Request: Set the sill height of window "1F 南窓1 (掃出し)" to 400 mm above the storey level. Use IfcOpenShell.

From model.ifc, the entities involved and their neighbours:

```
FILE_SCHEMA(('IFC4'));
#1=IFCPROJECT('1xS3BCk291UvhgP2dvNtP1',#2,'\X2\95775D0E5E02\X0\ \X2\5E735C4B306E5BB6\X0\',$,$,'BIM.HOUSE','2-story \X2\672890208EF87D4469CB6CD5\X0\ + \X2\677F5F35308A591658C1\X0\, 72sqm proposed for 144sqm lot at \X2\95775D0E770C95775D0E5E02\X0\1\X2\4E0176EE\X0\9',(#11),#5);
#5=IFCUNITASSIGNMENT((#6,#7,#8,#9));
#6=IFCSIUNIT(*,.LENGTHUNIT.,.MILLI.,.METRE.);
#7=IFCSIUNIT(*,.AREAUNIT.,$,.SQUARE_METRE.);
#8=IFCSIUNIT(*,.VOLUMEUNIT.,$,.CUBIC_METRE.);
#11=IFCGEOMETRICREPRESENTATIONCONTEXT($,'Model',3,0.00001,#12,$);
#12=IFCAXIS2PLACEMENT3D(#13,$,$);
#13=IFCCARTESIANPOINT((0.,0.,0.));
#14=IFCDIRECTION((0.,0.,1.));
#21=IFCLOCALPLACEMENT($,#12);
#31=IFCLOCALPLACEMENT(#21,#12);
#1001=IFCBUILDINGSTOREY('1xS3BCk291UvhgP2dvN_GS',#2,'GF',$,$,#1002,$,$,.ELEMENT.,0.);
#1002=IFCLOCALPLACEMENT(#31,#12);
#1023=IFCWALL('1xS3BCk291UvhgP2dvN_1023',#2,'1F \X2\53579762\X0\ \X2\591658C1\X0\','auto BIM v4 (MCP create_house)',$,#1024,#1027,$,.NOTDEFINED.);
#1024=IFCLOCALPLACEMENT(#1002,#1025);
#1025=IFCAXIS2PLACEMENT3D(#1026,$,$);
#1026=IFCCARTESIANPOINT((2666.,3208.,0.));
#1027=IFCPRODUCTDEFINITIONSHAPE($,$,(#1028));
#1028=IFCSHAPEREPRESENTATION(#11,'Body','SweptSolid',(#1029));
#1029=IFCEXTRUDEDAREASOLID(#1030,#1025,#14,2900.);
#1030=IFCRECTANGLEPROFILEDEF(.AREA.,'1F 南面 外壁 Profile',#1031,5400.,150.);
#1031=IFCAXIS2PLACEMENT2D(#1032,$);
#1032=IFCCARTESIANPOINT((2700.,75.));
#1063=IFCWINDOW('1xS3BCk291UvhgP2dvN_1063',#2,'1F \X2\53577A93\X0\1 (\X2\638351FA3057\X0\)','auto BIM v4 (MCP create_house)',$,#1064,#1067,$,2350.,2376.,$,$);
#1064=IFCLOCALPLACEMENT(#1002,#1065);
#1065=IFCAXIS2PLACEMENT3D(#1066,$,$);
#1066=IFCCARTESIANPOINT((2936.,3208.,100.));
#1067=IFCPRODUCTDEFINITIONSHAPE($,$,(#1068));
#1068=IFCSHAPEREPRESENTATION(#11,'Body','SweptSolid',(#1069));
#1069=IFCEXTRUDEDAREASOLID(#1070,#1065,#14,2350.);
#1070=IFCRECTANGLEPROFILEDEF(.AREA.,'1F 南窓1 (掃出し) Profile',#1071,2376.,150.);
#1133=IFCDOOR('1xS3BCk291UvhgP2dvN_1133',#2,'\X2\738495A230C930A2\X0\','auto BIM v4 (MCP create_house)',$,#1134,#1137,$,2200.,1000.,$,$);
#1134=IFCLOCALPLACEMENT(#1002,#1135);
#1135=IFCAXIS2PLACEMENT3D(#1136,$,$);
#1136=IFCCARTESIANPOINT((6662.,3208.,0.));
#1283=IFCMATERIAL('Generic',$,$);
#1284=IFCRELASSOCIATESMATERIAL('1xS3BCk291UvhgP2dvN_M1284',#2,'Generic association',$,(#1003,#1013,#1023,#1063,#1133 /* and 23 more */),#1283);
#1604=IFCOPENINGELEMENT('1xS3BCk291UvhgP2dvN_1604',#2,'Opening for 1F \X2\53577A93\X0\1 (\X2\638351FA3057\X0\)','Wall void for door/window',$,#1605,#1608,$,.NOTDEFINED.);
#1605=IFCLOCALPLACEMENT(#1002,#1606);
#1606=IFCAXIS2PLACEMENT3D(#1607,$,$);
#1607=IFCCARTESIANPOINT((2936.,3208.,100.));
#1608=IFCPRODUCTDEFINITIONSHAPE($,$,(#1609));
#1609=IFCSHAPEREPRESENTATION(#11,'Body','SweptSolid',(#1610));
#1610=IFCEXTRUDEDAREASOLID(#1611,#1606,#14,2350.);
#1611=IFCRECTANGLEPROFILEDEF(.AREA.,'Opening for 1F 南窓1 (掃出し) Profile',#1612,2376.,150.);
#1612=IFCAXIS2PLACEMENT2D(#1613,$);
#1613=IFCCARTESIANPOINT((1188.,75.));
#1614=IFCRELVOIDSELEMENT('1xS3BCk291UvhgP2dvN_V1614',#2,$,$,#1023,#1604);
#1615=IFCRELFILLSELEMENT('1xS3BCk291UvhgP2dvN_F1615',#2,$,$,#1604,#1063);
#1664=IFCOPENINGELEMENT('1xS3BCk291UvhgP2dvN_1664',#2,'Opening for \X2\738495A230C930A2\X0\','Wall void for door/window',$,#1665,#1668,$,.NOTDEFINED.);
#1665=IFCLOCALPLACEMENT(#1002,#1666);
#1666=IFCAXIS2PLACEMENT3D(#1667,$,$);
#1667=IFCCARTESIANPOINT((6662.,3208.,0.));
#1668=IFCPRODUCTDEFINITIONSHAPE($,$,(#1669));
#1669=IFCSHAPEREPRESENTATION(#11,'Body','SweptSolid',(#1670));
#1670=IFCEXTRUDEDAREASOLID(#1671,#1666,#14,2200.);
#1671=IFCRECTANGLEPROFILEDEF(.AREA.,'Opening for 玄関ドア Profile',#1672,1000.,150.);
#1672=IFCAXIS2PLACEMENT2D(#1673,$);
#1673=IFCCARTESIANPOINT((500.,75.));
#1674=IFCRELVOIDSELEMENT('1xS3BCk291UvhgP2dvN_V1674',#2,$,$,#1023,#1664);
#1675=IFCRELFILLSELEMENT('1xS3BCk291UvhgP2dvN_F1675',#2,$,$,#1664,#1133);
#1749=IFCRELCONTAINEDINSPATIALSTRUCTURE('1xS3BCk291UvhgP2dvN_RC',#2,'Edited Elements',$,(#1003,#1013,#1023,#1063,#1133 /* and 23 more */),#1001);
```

```python
import numpy as np
import ifcopenshell
import ifcopenshell.api.geometry
import ifcopenshell.geom
import ifcopenshell.util.element
import ifcopenshell.util.placement
import ifcopenshell.util.shape
import ifcopenshell.util.unit

model = ifcopenshell.open("model.ifc")
unit_scale = ifcopenshell.util.unit.calculate_unit_scale(model)

window = model.by_guid("1xS3BCk291UvhgP2dvN_1063")
opening = window.FillsVoids[0].RelatingOpeningElement
storey = ifcopenshell.util.element.get_container(window, ifc_class="IfcBuildingStorey")
level = ifcopenshell.util.placement.get_local_placement(storey.ObjectPlacement)[2, 3]

# The opening's origin need not be at the sill, so measure its lowest point.
shape = ifcopenshell.geom.create_shape(ifcopenshell.geom.settings(), opening)
bottom = ifcopenshell.util.shape.get_shape_bottom_elevation(shape, shape.geometry) / unit_scale
dz = level + 400.0 - bottom

shift = np.array([0.0, 0.0, dz])
# The window is not placed relative to its opening, so move both.
for product in (opening, window):
    matrix = ifcopenshell.util.placement.get_local_placement(product.ObjectPlacement)
    matrix[:3, 3] += shift
    ifcopenshell.api.geometry.edit_object_placement(model, product=product, matrix=matrix, is_si=False)

print(f"moved by {dz * unit_scale:+.3f} m")

model.write("model_updated.ifc")
```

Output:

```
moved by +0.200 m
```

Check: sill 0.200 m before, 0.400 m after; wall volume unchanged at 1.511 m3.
